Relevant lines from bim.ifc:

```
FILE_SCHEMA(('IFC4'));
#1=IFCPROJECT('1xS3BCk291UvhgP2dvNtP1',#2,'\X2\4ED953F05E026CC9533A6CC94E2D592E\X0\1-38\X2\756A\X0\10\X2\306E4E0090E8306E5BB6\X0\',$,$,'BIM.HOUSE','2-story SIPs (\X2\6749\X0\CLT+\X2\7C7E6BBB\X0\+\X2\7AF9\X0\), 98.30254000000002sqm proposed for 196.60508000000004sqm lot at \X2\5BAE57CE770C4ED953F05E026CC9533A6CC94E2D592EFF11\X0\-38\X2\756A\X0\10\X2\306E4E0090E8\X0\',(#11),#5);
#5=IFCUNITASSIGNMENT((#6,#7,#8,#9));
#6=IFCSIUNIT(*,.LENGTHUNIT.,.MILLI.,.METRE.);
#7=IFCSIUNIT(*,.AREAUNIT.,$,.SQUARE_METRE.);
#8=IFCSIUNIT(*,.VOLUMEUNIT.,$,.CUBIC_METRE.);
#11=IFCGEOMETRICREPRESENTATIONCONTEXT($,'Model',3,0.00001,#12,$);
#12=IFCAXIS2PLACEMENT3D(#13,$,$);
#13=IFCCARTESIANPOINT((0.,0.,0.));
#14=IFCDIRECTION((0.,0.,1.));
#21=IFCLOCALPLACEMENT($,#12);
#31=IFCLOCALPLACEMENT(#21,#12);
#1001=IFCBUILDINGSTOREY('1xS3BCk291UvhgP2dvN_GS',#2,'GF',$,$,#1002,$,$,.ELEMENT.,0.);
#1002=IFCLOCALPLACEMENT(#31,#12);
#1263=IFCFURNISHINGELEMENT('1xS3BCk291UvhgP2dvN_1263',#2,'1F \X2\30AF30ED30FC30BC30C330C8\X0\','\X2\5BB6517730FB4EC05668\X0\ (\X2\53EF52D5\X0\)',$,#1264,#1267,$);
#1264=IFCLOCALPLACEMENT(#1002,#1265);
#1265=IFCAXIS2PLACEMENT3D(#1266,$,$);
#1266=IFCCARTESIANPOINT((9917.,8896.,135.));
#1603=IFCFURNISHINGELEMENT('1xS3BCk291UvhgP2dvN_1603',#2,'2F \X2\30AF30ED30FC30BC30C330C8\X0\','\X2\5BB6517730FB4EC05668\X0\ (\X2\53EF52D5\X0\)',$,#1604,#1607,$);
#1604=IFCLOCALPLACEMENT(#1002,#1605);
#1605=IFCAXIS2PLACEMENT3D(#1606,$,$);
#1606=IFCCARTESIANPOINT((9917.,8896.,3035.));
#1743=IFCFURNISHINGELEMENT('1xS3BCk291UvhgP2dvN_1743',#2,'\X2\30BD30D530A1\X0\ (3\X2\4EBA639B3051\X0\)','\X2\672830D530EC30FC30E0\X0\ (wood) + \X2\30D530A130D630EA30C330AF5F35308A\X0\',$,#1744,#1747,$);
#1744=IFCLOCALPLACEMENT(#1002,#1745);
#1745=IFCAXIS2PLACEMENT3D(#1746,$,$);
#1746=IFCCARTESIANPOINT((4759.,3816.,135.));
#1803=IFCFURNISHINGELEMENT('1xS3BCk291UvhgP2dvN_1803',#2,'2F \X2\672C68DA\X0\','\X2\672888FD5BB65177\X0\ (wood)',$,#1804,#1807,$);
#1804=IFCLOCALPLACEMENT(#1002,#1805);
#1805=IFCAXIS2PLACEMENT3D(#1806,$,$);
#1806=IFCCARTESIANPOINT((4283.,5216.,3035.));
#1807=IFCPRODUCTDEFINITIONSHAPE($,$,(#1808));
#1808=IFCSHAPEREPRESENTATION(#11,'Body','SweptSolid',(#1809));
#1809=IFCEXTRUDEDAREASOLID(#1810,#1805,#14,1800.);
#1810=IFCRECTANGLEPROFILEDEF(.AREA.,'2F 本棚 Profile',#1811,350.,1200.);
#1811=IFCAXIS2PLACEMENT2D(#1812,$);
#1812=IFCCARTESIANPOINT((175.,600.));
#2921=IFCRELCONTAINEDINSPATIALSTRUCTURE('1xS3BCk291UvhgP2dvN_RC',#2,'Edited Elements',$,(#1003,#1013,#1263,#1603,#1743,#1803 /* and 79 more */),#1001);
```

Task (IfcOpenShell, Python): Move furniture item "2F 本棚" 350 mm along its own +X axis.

```python
import ifcopenshell
import ifcopenshell.api.geometry
import ifcopenshell.util.placement
import ifcopenshell.util.unit

model = ifcopenshell.open("bim.ifc")
unit_scale = ifcopenshell.util.unit.calculate_unit_scale(model)

item = model.by_guid("1xS3BCk291UvhgP2dvN_1803")
matrix = ifcopenshell.util.placement.get_local_placement(item.ObjectPlacement)
matrix[:3, 3] += matrix[:3, 0] * 0.35 / unit_scale
ifcopenshell.api.geometry.edit_object_placement(model, product=item, matrix=matrix, is_si=False)

print(ifcopenshell.util.placement.get_local_placement(item.ObjectPlacement).round(3) + 0.0)

model.write("bim_updated.ifc")
```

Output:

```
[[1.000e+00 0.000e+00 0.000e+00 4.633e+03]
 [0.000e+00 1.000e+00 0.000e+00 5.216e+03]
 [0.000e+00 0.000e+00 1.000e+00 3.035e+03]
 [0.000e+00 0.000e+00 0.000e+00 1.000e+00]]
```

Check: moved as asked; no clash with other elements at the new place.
